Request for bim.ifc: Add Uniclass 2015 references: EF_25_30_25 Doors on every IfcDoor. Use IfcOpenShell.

First a look at what the model holds.

```python
import ifcopenshell

model = ifcopenshell.open("bim.ifc")
print(model.schema)
print("classifications:", [c.Name for c in model.by_type("IfcClassification")])
for ifc_class in ("IfcDoor", "IfcRoof", "IfcStair", "IfcWall", "IfcWindow"):
    print(ifc_class, len(model.by_type(ifc_class)))
```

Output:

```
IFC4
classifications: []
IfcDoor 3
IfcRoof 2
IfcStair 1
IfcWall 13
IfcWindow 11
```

```python
import ifcopenshell
import ifcopenshell.api.classification

model = ifcopenshell.open("bim.ifc")

system = ifcopenshell.api.classification.add_classification(model, classification="Uniclass 2015")

codes = {
    "IfcDoor": ("EF_25_30_25", "Doors"),
}
for ifc_class, (code, name) in codes.items():
    products = model.by_type(ifc_class)
    ifcopenshell.api.classification.add_reference(
        model, products=products, classification=system, identification=code, name=name
    )
    print(code, len(products))

model.write("bim_edited.ifc")
```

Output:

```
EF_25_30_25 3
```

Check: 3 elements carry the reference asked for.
